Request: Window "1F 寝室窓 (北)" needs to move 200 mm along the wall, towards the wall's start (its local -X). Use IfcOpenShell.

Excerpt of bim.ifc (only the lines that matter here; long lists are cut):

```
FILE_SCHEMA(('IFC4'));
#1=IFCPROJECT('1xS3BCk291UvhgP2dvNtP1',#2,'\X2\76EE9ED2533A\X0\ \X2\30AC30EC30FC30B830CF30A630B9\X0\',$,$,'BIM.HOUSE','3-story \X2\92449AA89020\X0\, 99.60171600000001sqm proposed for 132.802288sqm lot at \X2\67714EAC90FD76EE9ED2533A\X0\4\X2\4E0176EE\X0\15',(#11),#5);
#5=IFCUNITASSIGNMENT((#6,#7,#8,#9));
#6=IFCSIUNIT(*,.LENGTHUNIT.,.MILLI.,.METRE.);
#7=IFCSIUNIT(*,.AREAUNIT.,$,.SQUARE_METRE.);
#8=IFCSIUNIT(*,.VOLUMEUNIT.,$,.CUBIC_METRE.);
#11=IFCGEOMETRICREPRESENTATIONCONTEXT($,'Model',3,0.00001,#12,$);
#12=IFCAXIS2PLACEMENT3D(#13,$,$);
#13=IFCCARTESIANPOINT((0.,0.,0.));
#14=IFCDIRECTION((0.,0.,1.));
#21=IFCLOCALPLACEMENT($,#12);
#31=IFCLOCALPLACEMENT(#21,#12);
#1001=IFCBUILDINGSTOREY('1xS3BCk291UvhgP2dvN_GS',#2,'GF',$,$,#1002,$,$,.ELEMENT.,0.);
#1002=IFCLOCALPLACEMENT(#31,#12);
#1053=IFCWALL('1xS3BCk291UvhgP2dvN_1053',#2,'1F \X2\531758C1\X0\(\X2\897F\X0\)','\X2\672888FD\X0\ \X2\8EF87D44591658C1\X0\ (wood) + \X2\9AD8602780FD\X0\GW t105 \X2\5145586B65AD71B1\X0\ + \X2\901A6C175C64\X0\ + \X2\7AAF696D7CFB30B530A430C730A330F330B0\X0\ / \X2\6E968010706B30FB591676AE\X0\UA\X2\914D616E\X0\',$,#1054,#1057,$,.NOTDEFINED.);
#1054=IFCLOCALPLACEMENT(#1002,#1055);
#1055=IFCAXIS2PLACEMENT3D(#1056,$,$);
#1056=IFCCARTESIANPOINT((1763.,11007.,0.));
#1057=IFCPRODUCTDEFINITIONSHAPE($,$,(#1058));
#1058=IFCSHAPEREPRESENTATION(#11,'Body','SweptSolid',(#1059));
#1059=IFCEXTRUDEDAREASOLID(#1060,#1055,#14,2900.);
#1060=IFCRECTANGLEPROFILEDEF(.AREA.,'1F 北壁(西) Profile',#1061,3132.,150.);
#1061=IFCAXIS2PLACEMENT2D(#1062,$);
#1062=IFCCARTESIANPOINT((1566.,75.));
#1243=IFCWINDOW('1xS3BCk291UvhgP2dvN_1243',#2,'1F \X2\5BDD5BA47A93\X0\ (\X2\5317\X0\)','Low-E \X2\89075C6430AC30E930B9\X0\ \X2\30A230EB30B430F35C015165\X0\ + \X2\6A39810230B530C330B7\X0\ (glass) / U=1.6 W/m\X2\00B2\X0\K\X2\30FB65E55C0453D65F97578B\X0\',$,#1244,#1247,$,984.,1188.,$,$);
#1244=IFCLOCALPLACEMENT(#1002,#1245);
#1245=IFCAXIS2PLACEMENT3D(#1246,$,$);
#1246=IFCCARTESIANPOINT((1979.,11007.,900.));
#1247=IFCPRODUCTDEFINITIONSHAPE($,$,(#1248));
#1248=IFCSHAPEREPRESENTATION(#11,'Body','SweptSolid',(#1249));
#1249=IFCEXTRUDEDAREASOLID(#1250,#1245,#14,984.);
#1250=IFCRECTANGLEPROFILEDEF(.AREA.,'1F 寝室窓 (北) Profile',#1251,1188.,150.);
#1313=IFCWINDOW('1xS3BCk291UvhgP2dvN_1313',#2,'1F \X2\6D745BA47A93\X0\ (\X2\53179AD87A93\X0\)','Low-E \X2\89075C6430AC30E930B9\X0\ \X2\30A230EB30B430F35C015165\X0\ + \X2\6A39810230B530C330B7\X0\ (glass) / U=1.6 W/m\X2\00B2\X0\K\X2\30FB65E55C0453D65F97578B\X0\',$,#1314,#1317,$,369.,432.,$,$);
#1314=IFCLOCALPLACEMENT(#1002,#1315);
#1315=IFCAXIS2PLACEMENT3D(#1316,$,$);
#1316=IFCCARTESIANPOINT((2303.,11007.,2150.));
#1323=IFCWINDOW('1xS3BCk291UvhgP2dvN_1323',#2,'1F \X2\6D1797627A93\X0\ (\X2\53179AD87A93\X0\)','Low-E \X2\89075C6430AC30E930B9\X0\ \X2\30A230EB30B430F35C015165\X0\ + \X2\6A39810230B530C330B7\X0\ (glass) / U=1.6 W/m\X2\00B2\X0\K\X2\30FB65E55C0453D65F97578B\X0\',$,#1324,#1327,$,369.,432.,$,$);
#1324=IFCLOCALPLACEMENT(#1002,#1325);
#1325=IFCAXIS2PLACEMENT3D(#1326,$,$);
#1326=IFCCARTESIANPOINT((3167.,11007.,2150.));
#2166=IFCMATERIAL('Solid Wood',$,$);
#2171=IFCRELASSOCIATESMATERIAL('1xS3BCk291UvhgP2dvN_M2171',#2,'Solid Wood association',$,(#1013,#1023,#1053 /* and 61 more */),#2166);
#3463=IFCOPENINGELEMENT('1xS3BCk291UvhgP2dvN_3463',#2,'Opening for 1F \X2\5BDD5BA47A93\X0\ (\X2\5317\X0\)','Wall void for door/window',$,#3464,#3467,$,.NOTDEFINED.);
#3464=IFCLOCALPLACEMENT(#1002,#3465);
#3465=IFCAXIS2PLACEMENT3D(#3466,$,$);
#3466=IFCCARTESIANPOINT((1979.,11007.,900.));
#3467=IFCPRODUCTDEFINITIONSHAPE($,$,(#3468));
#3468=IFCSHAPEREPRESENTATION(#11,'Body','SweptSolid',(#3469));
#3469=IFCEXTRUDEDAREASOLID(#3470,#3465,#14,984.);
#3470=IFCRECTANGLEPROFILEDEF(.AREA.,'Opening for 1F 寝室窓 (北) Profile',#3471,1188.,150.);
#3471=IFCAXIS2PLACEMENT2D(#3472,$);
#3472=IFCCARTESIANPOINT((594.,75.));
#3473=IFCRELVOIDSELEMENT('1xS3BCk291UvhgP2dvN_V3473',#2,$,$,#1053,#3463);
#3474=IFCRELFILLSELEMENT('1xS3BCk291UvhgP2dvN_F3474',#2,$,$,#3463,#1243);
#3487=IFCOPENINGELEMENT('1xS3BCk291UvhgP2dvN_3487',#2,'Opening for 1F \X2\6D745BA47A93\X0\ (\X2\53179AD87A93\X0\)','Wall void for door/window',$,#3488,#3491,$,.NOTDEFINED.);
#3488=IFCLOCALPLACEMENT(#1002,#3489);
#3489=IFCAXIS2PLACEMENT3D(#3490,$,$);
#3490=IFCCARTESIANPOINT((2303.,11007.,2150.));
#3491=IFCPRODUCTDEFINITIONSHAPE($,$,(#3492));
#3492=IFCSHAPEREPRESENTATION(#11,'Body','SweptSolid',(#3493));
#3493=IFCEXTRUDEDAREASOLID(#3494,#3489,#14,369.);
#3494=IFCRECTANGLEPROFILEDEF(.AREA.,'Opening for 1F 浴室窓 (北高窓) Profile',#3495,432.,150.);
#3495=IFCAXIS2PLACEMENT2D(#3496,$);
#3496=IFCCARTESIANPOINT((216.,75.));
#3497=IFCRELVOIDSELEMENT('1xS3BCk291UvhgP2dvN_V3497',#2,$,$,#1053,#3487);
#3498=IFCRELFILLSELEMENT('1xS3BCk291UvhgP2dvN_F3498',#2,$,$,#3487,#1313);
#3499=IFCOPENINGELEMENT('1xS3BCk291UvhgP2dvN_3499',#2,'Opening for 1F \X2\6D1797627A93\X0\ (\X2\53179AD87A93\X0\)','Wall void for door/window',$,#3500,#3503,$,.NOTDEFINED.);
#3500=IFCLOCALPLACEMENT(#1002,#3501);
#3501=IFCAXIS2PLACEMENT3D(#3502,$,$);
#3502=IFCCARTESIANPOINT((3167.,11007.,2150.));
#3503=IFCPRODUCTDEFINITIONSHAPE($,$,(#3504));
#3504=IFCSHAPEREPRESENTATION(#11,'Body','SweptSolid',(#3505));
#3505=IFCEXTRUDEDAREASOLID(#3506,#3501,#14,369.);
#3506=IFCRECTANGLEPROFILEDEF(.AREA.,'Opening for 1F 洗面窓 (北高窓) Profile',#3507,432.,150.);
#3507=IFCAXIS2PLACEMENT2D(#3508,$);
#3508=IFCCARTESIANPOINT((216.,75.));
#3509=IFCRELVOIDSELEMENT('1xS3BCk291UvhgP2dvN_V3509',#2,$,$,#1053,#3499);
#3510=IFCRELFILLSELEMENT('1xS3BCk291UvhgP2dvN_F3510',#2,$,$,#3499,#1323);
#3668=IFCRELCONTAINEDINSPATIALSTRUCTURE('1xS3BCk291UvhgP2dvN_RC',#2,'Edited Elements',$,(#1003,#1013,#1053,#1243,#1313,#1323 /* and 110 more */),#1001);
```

```python
import ifcopenshell
import ifcopenshell.api.geometry
import ifcopenshell.util.placement

model = ifcopenshell.open("bim.ifc")

window = model.by_guid("1xS3BCk291UvhgP2dvN_1243")
opening = window.FillsVoids[0].RelatingOpeningElement
wall = opening.VoidsElements[0].RelatingBuildingElement

wall_matrix = ifcopenshell.util.placement.get_local_placement(wall.ObjectPlacement)
shift = wall_matrix[:3, 0] * -200.0
before = ifcopenshell.util.placement.get_local_placement(window.ObjectPlacement)[:3, 3].copy()

# The window is not placed relative to its opening, so move both.
for product in (opening, window):
    matrix = ifcopenshell.util.placement.get_local_placement(product.ObjectPlacement)
    matrix[:3, 3] += shift
    ifcopenshell.api.geometry.edit_object_placement(model, product=product, matrix=matrix, is_si=False)

after = ifcopenshell.util.placement.get_local_placement(window.ObjectPlacement)[:3, 3]
print("window moved by", (after - before).round(3) + 0.0)

model.write("bim_edited.ifc")
```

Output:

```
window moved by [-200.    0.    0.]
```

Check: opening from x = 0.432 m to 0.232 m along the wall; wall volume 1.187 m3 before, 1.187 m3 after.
